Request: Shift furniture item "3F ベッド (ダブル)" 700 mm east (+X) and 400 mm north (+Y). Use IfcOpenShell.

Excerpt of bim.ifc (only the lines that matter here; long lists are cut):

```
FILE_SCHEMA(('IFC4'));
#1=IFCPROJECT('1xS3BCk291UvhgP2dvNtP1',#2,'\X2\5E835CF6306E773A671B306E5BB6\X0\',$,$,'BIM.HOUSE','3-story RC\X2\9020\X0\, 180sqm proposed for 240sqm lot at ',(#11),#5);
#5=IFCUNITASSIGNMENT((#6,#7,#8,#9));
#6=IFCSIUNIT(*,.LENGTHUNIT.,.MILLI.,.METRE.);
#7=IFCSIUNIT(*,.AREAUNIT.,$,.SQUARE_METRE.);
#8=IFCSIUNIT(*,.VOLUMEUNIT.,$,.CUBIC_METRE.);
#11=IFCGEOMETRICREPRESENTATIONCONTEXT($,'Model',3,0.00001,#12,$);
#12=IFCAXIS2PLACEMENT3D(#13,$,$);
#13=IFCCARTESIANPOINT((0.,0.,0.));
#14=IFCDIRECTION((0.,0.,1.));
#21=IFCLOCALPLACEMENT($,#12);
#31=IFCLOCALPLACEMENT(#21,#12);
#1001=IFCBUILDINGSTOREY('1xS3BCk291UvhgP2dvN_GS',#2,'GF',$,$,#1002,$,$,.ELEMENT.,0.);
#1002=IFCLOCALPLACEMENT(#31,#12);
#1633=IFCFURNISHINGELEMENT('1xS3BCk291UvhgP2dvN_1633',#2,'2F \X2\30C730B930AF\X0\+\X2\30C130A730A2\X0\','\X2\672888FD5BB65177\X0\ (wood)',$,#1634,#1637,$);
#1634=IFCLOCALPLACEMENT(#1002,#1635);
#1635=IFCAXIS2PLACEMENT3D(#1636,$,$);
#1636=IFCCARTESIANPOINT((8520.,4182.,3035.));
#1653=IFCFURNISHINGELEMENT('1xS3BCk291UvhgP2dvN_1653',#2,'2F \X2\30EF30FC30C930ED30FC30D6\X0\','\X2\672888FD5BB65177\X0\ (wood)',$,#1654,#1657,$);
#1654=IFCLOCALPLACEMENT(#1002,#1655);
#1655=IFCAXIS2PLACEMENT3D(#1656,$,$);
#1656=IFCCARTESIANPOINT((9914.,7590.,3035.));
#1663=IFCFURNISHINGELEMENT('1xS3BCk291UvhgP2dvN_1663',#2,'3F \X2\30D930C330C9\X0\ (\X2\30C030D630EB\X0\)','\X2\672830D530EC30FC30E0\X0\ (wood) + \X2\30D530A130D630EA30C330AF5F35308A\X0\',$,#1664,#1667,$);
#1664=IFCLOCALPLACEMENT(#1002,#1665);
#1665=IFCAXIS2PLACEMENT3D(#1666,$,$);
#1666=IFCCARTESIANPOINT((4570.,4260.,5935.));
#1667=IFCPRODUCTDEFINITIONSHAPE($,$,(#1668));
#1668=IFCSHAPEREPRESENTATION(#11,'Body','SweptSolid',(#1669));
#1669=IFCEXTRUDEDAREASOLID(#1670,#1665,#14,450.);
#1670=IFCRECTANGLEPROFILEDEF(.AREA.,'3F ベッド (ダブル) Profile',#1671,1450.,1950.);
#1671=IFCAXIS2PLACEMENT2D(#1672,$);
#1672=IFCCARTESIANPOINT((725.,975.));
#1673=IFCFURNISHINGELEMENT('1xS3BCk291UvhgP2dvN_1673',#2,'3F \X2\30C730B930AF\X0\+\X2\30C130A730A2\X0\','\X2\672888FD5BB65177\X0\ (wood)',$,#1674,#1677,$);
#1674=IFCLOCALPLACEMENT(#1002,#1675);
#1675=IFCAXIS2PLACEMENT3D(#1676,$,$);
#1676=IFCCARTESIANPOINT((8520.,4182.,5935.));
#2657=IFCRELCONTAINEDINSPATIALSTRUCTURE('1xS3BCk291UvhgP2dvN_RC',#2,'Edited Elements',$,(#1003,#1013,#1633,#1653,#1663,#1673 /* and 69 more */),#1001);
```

```python
import ifcopenshell
import ifcopenshell.api.geometry
import ifcopenshell.util.placement
import ifcopenshell.util.unit

model = ifcopenshell.open("bim.ifc")
unit_scale = ifcopenshell.util.unit.calculate_unit_scale(model)

item = model.by_id(1663)
matrix = ifcopenshell.util.placement.get_local_placement(item.ObjectPlacement)
matrix[0, 3] += 0.7 / unit_scale
matrix[1, 3] += 0.4 / unit_scale
ifcopenshell.api.geometry.edit_object_placement(model, product=item, matrix=matrix, is_si=False)

print(ifcopenshell.util.placement.get_local_placement(item.ObjectPlacement).round(3) + 0.0)

model.write("bim_rev.ifc")
```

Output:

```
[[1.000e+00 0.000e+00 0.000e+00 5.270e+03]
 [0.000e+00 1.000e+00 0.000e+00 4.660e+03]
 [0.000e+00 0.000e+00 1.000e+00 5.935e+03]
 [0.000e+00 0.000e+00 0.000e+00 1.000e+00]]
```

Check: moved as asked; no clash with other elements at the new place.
